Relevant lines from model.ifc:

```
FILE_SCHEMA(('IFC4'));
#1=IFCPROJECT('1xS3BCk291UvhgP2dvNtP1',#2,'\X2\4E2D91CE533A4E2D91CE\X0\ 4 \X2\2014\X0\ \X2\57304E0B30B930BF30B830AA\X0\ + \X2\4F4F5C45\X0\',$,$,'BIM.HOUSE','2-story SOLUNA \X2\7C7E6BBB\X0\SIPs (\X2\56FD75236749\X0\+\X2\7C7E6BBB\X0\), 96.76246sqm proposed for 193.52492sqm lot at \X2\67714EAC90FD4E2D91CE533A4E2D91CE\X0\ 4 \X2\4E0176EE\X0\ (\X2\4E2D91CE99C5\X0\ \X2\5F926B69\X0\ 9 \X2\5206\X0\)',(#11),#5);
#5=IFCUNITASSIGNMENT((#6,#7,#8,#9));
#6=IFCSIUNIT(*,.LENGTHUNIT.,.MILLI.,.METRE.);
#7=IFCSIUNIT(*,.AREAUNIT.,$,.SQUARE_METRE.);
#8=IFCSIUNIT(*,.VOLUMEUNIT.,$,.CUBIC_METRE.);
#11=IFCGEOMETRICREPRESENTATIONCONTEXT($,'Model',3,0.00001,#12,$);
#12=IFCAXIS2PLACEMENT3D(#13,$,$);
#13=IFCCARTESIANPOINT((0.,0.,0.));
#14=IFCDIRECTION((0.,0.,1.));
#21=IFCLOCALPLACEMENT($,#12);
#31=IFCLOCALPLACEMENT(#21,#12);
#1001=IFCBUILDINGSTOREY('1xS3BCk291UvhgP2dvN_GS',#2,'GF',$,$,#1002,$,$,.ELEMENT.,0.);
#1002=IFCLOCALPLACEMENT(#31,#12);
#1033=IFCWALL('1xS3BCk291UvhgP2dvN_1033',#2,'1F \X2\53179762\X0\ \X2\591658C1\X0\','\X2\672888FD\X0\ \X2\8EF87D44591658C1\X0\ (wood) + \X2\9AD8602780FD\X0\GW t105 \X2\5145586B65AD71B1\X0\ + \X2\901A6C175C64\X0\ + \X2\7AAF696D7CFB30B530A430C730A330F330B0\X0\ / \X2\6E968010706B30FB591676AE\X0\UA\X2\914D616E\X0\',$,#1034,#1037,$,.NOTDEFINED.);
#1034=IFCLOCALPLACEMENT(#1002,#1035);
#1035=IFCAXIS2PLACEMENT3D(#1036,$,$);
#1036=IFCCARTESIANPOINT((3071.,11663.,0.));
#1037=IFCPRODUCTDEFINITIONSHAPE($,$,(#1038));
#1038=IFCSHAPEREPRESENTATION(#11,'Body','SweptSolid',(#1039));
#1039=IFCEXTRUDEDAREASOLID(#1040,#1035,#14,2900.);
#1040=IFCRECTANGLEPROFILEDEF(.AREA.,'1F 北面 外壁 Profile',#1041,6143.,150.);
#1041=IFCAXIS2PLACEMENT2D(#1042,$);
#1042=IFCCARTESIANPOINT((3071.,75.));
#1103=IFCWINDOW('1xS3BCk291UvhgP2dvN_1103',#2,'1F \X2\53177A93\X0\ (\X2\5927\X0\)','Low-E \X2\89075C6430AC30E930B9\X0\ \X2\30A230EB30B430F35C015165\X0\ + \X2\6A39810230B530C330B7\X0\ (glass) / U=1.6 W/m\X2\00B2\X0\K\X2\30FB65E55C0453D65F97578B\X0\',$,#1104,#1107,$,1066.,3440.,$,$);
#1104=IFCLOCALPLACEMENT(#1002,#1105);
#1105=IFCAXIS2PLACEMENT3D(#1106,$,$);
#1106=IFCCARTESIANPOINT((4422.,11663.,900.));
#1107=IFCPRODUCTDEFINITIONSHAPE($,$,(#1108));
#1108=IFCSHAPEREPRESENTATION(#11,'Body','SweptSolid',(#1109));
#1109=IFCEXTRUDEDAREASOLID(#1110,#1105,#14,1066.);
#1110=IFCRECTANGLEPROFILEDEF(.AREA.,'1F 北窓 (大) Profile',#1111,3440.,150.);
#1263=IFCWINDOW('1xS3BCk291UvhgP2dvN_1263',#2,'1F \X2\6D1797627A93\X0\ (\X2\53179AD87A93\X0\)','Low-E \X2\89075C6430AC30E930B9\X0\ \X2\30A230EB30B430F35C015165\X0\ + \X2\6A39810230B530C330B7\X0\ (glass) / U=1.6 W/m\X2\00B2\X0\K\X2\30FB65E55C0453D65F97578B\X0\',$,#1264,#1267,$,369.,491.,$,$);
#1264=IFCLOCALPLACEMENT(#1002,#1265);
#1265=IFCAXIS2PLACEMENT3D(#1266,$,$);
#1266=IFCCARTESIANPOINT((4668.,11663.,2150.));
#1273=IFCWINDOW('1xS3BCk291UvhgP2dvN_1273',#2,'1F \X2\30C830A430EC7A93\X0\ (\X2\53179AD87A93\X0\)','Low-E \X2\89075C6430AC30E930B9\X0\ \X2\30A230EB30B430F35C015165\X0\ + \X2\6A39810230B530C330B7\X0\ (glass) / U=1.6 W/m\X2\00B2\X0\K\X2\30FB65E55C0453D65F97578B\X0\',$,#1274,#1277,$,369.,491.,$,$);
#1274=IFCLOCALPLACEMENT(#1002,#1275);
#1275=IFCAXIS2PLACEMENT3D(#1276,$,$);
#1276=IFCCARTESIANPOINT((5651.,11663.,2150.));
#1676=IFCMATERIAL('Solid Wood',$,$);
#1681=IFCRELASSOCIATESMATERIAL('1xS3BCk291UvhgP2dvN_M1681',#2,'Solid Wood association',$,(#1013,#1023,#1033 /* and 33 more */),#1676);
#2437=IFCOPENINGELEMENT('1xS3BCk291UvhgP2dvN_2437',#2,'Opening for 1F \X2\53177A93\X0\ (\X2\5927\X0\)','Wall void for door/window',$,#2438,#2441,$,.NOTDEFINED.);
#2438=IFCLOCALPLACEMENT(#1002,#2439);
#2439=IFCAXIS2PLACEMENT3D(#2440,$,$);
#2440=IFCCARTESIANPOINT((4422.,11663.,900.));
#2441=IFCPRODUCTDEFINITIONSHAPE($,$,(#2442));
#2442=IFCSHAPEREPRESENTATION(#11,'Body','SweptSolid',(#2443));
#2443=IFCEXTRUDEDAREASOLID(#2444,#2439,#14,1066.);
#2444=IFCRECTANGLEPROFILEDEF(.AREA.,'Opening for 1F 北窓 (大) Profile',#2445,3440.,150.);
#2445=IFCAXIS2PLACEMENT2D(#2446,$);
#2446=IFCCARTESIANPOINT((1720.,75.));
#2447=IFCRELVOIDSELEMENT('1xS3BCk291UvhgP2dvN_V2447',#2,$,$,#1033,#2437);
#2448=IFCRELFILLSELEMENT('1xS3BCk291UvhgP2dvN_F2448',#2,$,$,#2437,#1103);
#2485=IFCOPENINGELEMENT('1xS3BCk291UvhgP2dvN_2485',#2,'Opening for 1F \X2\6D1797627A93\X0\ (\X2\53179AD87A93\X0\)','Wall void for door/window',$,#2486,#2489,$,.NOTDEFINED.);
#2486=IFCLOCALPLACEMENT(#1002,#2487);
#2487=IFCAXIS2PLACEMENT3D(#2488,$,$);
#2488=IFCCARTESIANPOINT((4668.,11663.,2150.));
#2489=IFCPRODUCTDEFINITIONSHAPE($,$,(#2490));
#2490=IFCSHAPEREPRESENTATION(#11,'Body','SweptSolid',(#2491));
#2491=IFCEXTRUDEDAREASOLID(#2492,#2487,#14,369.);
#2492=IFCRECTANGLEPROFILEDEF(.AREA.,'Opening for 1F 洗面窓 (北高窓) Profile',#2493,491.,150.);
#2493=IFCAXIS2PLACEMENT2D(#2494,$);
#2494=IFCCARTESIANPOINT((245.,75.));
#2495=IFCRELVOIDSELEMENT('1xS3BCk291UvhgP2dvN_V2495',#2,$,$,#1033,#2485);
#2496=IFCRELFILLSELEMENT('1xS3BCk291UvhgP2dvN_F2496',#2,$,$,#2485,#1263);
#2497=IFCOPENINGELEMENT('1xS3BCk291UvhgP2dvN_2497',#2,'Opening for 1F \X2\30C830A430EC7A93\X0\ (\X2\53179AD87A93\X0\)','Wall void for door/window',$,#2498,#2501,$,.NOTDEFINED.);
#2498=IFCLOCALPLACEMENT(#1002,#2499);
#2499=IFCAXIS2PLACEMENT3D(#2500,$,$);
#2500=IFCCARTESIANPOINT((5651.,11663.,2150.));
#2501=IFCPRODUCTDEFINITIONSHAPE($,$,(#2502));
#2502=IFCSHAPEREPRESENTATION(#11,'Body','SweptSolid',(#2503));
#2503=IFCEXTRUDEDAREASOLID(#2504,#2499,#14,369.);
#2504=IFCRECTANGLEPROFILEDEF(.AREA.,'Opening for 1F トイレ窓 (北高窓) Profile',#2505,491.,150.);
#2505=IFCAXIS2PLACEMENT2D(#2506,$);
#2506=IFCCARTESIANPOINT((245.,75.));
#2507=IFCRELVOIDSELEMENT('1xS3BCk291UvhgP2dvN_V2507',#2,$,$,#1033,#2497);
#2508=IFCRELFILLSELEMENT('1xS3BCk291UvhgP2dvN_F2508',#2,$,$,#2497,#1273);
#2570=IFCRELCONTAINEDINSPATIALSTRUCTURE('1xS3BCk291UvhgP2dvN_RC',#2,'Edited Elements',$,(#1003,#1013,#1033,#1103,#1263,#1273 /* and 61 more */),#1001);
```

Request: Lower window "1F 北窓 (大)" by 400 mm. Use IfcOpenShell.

```python
import numpy as np
import ifcopenshell
import ifcopenshell.api.geometry
import ifcopenshell.util.placement
import ifcopenshell.util.unit

model = ifcopenshell.open("model.ifc")
unit_scale = ifcopenshell.util.unit.calculate_unit_scale(model)

window = model.by_guid("1xS3BCk291UvhgP2dvN_1103")
opening = window.FillsVoids[0].RelatingOpeningElement
dz = -0.4 / unit_scale

shift = np.array([0.0, 0.0, dz])
# The window is not placed relative to its opening, so move both.
for product in (opening, window):
    matrix = ifcopenshell.util.placement.get_local_placement(product.ObjectPlacement)
    matrix[:3, 3] += shift
    ifcopenshell.api.geometry.edit_object_placement(model, product=product, matrix=matrix, is_si=False)

print(f"moved by {dz * unit_scale:+.3f} m")

model.write("model_updated.ifc")
```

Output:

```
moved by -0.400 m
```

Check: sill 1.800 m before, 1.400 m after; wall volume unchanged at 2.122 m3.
